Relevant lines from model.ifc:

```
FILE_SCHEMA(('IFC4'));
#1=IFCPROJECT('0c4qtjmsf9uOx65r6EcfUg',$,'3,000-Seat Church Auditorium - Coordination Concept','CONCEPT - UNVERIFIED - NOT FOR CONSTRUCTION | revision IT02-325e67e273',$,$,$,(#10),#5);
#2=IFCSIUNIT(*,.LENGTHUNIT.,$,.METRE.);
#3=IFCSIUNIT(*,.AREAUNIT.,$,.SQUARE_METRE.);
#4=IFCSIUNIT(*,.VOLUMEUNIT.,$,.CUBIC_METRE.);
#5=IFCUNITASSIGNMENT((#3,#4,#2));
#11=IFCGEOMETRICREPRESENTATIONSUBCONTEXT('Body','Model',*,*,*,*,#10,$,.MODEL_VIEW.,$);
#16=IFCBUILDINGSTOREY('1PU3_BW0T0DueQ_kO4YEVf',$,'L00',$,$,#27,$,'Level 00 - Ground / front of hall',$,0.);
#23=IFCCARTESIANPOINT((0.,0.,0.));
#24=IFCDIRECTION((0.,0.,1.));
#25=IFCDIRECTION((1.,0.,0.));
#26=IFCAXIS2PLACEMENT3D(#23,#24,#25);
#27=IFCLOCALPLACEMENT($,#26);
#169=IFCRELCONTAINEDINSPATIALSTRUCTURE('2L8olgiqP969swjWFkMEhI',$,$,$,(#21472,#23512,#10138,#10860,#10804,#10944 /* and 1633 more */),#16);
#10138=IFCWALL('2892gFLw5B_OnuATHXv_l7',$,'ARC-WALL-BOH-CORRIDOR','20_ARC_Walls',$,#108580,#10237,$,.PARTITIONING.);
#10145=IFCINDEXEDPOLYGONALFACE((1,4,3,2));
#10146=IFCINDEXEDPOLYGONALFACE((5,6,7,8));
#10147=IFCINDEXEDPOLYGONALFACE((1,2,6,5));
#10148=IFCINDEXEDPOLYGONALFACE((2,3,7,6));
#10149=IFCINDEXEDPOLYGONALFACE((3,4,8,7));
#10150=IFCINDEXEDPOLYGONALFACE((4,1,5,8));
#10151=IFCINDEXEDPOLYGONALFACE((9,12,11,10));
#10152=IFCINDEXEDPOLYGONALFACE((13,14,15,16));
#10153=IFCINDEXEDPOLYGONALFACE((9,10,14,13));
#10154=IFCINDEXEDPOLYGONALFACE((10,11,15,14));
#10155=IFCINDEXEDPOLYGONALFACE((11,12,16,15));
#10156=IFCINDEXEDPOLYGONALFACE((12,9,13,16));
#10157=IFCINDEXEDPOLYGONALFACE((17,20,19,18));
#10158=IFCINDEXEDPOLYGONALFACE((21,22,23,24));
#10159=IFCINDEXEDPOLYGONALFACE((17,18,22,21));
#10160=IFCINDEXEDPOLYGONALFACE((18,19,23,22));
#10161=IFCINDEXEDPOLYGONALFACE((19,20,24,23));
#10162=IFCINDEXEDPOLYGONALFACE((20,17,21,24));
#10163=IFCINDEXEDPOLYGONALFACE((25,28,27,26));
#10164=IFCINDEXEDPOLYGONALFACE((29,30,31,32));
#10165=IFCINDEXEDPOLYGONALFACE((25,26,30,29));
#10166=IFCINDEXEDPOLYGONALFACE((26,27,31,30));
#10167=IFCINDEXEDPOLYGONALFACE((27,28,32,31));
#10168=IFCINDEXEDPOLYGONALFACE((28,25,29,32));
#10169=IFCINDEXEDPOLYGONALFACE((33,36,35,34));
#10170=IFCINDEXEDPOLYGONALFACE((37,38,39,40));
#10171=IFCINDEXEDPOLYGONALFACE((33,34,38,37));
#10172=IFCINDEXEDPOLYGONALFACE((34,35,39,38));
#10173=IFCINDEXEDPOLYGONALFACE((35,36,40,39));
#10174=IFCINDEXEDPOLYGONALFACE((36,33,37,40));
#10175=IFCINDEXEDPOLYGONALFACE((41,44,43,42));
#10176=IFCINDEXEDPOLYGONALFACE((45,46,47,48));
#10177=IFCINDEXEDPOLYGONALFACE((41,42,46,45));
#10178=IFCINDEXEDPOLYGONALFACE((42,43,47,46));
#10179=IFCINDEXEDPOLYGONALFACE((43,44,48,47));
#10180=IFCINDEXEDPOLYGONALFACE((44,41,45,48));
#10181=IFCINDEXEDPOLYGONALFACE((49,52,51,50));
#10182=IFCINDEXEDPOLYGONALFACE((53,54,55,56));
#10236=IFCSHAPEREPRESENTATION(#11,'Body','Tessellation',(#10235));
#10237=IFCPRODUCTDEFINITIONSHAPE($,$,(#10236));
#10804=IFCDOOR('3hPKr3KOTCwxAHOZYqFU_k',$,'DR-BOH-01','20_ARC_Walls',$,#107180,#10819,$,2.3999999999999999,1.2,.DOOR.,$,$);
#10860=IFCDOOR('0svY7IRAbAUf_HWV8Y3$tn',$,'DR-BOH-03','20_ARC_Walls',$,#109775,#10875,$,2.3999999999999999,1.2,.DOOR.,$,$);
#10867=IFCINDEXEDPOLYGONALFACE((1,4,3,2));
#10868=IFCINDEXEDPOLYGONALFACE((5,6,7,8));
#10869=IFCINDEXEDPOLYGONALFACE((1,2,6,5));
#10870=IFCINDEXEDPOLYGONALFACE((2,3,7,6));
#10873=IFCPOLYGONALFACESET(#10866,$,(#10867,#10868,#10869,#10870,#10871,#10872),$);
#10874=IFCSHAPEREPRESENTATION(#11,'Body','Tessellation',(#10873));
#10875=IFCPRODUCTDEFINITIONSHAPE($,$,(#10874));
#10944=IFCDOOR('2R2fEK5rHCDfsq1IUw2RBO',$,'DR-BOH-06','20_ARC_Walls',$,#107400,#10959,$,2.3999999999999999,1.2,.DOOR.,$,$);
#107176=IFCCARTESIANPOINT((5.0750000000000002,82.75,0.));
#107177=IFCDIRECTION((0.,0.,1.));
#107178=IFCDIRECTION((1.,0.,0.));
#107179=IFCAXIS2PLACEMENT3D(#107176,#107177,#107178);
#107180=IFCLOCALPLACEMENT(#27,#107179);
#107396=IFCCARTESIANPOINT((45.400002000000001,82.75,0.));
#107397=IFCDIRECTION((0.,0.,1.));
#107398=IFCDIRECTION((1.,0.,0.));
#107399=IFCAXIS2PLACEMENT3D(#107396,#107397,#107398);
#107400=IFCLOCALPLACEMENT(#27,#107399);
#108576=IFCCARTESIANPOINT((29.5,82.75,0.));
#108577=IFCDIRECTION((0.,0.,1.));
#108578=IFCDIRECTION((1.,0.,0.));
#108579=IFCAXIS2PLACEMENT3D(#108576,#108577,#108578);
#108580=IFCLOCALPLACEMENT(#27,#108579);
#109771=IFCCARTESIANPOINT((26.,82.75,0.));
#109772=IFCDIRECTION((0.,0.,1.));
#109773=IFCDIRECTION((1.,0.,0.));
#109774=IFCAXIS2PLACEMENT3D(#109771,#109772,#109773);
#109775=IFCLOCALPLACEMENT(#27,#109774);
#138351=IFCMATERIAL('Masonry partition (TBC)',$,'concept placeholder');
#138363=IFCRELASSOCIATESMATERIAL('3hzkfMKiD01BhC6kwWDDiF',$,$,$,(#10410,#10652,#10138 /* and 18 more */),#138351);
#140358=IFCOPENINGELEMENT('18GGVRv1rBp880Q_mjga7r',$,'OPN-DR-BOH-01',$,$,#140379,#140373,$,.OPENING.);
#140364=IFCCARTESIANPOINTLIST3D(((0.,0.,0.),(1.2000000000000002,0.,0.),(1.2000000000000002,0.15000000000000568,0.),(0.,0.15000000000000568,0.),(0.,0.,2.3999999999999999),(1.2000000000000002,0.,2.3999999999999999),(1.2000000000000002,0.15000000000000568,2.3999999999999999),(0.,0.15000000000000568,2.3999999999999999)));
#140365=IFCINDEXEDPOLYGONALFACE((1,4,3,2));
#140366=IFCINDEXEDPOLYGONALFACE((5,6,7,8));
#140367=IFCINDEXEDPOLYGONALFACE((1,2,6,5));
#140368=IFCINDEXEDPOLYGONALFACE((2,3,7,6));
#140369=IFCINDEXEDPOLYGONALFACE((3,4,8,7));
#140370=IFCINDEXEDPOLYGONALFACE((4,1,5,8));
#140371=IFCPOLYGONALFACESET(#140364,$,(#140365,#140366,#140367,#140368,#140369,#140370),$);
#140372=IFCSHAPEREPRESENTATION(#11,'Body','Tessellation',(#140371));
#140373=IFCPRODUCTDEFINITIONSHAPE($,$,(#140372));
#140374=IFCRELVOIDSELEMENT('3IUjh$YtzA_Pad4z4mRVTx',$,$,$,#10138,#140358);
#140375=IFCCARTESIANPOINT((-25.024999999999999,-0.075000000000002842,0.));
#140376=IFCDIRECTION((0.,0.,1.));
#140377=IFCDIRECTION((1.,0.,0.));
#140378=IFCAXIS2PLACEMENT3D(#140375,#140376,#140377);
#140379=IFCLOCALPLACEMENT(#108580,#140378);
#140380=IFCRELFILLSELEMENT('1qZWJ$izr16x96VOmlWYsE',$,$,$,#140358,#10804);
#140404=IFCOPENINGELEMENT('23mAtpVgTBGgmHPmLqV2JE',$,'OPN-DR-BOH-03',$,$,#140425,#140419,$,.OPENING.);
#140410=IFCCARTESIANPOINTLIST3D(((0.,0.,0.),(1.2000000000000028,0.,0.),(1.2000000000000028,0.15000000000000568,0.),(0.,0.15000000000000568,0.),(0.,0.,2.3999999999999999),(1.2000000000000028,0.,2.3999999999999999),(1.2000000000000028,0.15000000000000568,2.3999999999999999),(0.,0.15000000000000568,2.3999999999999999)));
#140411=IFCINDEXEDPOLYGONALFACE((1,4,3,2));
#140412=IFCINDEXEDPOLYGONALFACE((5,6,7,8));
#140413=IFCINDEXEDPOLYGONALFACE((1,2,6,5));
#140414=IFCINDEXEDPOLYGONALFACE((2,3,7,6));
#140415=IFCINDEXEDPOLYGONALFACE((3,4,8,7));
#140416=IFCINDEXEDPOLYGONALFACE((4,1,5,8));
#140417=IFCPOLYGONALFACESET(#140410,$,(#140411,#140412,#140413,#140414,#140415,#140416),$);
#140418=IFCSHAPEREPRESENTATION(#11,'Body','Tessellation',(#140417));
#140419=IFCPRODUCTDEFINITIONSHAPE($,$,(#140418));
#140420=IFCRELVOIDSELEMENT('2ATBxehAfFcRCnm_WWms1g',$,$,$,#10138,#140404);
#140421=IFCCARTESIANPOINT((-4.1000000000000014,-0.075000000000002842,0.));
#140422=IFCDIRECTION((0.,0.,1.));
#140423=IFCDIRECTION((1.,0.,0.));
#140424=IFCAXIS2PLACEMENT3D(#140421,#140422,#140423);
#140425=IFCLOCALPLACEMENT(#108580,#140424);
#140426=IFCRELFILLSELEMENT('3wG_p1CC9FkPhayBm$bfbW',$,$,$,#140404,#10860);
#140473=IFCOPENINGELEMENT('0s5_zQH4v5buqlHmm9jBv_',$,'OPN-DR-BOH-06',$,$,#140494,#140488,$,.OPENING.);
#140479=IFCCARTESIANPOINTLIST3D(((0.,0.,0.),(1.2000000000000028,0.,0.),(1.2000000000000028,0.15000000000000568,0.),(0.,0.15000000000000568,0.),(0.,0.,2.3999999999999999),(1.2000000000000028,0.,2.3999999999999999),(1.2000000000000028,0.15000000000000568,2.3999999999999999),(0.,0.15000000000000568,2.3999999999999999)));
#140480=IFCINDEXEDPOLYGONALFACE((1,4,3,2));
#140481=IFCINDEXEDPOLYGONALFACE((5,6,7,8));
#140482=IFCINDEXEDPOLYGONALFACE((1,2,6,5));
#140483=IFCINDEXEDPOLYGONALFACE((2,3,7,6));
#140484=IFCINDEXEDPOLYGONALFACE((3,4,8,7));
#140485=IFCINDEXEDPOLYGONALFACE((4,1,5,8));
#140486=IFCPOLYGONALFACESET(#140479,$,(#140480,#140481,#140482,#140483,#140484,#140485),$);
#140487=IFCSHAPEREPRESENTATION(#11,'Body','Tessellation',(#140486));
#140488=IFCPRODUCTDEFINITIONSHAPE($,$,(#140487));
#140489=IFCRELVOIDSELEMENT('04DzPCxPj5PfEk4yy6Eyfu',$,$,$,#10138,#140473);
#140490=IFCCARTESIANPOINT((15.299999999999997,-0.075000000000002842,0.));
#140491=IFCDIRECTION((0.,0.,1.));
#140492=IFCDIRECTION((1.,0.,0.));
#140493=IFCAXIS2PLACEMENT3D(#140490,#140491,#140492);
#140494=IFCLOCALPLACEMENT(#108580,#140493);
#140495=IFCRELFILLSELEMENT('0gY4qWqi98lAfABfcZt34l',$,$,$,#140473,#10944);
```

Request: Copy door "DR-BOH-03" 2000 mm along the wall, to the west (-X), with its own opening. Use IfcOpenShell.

```python
import ifcopenshell
import ifcopenshell.api.feature
import ifcopenshell.api.geometry
import ifcopenshell.api.root
import ifcopenshell.geom
import ifcopenshell.util.element
import ifcopenshell.util.placement
import ifcopenshell.util.shape
import ifcopenshell.util.unit

model = ifcopenshell.open("model.ifc")
unit_scale = ifcopenshell.util.unit.calculate_unit_scale(model)
settings = ifcopenshell.geom.settings()


def volume(element):
    """Net volume in cubic metres, openings subtracted."""
    shape = ifcopenshell.geom.create_shape(settings, element)
    return ifcopenshell.util.shape.get_volume(shape.geometry)


door = model.by_guid("0svY7IRAbAUf_HWV8Y3$tn")
opening = door.FillsVoids[0].RelatingOpeningElement
wall = opening.VoidsElements[0].RelatingBuildingElement
before = volume(wall)
shift = ifcopenshell.util.placement.get_local_placement(wall.ObjectPlacement)[:3, 0] * -2 / unit_scale

# copy_class copies the void relationship, type, container and properties, but no geometry.
new_opening = ifcopenshell.api.root.copy_class(model, product=opening)
new_opening.Representation = ifcopenshell.util.element.copy_deep(
    model, opening.Representation, exclude=["IfcGeometricRepresentationContext", "IfcRepresentationMap"]
)
new_door = ifcopenshell.api.root.copy_class(model, product=door)
new_door.Representation = ifcopenshell.util.element.copy_deep(
    model, door.Representation, exclude=["IfcGeometricRepresentationContext", "IfcRepresentationMap"]
)
ifcopenshell.api.feature.add_filling(model, opening=new_opening, element=new_door)

for old, new in ((opening, new_opening), (door, new_door)):
    matrix = ifcopenshell.util.placement.get_local_placement(old.ObjectPlacement)
    matrix[:3, 3] += shift
    ifcopenshell.api.geometry.edit_object_placement(model, product=new, matrix=matrix, is_si=False)

after = volume(wall)

print(f"wall volume {before:.3f} -> {after:.3f} m3")

model.write("model_updated.ifc")
```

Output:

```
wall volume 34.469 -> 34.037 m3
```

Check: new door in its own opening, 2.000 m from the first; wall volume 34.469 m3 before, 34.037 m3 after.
